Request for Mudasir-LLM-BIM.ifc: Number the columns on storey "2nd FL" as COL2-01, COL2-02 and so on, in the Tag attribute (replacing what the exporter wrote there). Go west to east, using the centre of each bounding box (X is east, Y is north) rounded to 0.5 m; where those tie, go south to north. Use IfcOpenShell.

First a look at what the model holds.

```python
import ifcopenshell
import ifcopenshell.util.element
import ifcopenshell.util.placement

model = ifcopenshell.open("Mudasir-LLM-BIM.ifc")
print(model.schema)
storey = next(s for s in model.by_type("IfcBuildingStorey") if s.Name == "2nd FL")
columns = [e for e in ifcopenshell.util.element.get_decomposition(storey) if e.is_a("IfcColumn")]
for e in sorted(columns, key=lambda e: e.id()):
    origin = ifcopenshell.util.placement.get_local_placement(e.ObjectPlacement)[:3, 3]
    print(e.id(), e.Tag, e.Name, origin.round(2) + 0.0, sep=" | ")
```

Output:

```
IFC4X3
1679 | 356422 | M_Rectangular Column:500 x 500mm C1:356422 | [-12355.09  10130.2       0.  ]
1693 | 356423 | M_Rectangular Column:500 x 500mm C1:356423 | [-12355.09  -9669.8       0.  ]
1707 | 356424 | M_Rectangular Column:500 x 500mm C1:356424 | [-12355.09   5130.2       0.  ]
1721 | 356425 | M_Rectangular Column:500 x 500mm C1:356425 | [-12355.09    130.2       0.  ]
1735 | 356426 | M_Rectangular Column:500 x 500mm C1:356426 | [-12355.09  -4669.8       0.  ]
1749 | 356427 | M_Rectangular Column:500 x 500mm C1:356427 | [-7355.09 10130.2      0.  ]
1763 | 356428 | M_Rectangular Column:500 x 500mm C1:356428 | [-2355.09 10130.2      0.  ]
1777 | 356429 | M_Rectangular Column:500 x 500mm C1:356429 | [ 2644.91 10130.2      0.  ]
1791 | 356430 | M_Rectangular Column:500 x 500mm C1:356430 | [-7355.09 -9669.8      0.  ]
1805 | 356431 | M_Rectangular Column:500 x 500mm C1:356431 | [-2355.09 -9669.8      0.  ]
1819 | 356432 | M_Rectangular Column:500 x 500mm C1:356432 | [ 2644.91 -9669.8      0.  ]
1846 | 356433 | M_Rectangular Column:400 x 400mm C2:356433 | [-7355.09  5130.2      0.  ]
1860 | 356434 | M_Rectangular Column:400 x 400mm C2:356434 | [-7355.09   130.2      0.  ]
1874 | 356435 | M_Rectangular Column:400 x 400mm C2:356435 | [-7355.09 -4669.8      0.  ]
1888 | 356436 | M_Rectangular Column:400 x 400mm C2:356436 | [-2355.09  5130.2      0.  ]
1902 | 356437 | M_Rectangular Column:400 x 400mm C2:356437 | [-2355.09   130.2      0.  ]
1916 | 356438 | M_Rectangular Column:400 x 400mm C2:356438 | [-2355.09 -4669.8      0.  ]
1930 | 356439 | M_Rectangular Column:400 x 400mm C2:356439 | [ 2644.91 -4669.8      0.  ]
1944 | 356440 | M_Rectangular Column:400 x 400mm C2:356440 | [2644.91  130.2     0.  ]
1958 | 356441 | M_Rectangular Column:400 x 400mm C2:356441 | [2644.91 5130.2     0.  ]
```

```python
import ifcopenshell
import ifcopenshell.geom
import ifcopenshell.util.element
import ifcopenshell.util.shape

model = ifcopenshell.open("Mudasir-LLM-BIM.ifc")
settings = ifcopenshell.geom.settings()
settings.set("use-world-coords", True)


def centre(element):
    shape = ifcopenshell.geom.create_shape(settings, element)
    return ifcopenshell.util.shape.get_bbox_centroid(shape.geometry)


storey = next(s for s in model.by_type("IfcBuildingStorey") if s.Name == "2nd FL")
columns = [e for e in ifcopenshell.util.element.get_decomposition(storey) if e.is_a("IfcColumn")]

# Insertion points can sit at a corner or the storey origin, so sort by the geometry (in metres).
centres = {e: centre(e) for e in columns}
columns.sort(key=lambda e: (round(centres[e][0] / 0.5), centres[e][1]))

for i, e in enumerate(columns, start=1):
    number = f"COL2-{i:02d}"
    e.Tag = number
    print(e.id(), number)

model.write("Mudasir-LLM-BIM_rev.ifc")
```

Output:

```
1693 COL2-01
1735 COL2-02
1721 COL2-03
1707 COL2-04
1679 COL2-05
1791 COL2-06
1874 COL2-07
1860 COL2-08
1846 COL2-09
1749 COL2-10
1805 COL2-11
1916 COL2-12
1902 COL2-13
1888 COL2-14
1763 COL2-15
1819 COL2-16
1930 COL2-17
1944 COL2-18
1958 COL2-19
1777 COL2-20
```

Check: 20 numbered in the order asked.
